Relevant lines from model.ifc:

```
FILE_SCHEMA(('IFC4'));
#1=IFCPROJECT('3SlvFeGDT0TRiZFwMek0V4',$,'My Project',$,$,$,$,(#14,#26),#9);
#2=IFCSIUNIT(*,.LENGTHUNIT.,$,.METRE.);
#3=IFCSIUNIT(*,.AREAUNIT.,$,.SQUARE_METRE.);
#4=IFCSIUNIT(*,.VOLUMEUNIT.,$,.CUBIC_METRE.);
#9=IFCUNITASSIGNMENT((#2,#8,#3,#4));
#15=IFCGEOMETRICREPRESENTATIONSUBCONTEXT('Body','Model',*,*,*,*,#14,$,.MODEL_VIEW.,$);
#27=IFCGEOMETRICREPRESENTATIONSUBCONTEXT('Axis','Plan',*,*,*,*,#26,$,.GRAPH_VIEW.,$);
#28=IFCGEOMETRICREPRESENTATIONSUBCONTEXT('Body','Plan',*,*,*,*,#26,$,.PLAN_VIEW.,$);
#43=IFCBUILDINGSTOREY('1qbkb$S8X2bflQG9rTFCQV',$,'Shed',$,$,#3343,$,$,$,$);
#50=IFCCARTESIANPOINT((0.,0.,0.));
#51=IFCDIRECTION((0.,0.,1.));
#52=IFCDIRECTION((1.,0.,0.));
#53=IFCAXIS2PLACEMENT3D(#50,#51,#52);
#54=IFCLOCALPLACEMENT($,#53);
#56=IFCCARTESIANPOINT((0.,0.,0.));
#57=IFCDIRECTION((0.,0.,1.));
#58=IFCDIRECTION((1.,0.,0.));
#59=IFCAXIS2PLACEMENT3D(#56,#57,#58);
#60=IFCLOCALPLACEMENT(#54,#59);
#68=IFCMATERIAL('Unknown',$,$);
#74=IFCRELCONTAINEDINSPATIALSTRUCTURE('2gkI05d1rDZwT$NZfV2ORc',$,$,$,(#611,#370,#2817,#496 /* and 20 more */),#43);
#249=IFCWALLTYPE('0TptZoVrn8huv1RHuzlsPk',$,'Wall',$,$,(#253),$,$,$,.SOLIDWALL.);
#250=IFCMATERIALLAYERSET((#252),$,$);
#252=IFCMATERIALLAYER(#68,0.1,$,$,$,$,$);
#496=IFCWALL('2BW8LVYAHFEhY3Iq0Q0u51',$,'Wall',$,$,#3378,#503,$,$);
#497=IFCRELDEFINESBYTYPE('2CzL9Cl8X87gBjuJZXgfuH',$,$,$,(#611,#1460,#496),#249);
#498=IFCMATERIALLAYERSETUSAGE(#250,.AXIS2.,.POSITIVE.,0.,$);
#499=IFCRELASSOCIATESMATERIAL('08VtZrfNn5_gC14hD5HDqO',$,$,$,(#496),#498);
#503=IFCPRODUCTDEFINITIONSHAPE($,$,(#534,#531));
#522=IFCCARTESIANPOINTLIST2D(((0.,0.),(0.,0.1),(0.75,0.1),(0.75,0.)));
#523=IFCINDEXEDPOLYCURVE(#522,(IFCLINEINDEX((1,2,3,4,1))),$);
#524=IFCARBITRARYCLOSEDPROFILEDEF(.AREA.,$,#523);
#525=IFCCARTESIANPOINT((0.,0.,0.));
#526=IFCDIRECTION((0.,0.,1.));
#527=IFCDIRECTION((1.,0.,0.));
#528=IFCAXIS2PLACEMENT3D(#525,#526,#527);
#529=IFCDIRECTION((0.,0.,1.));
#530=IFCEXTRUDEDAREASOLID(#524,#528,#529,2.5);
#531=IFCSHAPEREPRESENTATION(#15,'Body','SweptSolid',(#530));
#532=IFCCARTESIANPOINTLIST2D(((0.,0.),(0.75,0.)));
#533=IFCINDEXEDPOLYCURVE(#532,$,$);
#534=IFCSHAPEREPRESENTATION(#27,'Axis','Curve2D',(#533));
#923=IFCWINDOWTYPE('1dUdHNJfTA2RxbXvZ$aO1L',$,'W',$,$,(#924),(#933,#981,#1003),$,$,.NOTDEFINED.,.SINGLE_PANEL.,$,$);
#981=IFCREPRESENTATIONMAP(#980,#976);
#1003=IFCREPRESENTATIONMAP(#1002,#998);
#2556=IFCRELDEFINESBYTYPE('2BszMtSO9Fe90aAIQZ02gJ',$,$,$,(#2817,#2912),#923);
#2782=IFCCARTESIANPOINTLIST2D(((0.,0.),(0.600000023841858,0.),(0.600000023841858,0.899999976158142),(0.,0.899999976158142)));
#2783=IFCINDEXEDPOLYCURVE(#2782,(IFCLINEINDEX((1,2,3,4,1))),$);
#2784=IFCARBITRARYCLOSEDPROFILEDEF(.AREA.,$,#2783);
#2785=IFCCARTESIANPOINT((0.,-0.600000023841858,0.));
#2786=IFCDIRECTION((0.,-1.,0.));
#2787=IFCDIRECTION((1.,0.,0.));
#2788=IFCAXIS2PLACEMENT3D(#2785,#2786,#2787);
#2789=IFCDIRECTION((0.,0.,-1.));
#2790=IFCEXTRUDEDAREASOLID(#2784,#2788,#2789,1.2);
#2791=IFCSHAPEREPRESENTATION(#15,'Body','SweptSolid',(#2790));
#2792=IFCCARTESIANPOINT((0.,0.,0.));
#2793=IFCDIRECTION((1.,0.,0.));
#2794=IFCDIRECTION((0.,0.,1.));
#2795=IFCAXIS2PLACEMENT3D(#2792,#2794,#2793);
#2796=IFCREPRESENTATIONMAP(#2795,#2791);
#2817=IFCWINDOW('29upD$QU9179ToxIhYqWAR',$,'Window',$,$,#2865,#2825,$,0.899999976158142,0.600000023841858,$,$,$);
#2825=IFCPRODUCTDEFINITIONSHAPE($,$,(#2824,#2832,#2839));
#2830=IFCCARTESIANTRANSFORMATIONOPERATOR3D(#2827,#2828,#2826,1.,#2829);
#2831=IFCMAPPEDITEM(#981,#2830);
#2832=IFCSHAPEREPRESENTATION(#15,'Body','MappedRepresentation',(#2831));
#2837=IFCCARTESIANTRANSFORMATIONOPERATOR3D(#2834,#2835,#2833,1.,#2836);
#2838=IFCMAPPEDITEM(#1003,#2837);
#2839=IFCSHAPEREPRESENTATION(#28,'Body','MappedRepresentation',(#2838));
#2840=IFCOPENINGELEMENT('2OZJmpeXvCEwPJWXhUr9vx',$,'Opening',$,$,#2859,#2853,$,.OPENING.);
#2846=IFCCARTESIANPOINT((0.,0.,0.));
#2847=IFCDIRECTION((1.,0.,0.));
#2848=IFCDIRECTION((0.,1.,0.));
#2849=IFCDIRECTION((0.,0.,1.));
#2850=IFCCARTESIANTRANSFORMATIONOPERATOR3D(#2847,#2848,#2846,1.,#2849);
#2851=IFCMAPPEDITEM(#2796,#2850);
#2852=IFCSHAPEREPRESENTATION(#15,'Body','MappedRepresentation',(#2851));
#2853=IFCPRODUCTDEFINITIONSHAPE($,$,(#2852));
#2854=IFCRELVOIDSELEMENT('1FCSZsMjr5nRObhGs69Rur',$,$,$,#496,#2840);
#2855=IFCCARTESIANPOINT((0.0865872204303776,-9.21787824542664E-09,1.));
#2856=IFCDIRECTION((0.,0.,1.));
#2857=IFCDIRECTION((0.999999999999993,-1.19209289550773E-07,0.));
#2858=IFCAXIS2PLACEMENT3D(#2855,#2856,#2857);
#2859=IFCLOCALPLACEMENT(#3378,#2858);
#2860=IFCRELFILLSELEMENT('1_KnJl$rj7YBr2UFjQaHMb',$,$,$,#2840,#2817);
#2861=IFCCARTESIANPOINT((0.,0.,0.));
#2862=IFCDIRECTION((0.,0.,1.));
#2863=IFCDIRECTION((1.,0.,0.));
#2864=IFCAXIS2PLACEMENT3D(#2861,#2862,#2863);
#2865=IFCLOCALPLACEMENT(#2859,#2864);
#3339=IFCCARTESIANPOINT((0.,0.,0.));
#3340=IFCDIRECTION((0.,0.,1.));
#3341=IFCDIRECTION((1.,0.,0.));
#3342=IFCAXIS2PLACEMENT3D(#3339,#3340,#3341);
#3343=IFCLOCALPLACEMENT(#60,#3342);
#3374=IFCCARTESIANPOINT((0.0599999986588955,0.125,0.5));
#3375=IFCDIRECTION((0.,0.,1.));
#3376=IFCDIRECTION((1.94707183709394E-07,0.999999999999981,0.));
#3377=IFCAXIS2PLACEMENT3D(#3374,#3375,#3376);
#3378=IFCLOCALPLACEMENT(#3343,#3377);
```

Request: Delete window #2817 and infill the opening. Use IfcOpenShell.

```python
import ifcopenshell
import ifcopenshell.api.feature
import ifcopenshell.api.root
import ifcopenshell.geom
import ifcopenshell.util.shape

model = ifcopenshell.open("model.ifc")
settings = ifcopenshell.geom.settings()


def volume(element):
    """Net volume in cubic metres, openings subtracted."""
    shape = ifcopenshell.geom.create_shape(settings, element)
    return ifcopenshell.util.shape.get_volume(shape.geometry)


window = model.by_guid("29upD$QU9179ToxIhYqWAR")
opening = window.FillsVoids[0].RelatingOpeningElement
wall = opening.VoidsElements[0].RelatingBuildingElement
before = volume(wall)

ifcopenshell.api.root.remove_product(model, product=window)
ifcopenshell.api.feature.remove_feature(model, feature=opening)

after = volume(wall)

print(f"wall volume {before:.3f} -> {after:.3f} m3")

model.write("model_edited.ifc")
```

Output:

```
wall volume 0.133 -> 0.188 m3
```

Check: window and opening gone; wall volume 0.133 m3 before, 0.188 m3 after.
